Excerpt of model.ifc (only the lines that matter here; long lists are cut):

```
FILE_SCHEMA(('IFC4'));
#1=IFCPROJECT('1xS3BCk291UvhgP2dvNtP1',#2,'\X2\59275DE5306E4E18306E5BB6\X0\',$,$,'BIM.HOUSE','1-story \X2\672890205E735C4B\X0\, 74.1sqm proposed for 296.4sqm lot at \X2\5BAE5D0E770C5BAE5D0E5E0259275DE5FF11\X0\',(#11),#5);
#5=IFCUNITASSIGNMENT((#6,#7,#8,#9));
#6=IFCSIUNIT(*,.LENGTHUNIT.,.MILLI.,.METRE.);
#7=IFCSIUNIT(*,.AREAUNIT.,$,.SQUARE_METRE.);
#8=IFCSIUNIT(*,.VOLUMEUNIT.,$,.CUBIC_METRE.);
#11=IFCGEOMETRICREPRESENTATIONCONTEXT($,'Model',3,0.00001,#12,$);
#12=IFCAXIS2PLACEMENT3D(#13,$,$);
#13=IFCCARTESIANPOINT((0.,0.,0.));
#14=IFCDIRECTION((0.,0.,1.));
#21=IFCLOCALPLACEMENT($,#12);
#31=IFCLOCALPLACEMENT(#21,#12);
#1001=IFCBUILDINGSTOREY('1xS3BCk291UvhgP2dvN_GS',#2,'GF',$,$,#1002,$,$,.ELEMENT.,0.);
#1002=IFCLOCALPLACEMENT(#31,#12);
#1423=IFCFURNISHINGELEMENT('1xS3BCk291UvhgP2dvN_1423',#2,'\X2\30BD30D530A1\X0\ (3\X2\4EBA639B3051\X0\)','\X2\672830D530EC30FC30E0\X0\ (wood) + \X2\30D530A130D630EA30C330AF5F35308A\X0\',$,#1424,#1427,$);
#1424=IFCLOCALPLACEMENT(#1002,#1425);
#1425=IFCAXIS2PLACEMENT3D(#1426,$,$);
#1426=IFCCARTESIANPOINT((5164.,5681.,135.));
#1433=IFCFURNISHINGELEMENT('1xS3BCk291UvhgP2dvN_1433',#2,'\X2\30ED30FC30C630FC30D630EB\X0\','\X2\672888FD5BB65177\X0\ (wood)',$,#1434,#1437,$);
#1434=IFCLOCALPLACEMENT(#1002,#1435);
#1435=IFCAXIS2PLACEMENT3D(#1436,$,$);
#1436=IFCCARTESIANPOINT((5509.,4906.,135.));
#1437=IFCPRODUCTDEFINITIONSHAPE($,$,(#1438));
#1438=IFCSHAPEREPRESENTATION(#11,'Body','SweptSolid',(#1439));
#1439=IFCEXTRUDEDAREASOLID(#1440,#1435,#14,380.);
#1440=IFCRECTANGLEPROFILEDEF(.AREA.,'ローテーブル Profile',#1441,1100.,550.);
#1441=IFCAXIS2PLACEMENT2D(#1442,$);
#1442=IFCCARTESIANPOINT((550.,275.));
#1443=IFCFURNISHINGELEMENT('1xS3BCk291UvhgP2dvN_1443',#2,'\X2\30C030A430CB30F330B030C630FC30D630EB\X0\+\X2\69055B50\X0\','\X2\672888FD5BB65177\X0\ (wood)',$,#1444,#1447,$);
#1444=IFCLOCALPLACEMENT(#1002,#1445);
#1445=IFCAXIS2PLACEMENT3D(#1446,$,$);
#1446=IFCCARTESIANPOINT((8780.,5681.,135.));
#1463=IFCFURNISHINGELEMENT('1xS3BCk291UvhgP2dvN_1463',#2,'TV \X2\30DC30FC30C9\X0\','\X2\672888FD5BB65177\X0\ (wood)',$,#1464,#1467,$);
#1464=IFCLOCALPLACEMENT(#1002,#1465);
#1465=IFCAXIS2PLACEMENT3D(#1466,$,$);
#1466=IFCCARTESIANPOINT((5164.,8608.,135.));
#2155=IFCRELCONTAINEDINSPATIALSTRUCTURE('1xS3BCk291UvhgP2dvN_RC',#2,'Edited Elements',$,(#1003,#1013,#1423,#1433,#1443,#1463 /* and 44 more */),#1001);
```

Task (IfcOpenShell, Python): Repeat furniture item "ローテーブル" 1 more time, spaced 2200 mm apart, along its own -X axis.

```python
import ifcopenshell
import ifcopenshell.api.geometry
import ifcopenshell.api.root
import ifcopenshell.util.element
import ifcopenshell.util.placement

model = ifcopenshell.open("model.ifc")


def reuse_history(source, copy):
    """copy_class also copies each property set's owner history, people and application; keep the originals."""
    for rel in copy.IsDefinedBy:
        if rel.is_a("IfcRelDefinesByProperties") and (history := rel.RelatingPropertyDefinition.OwnerHistory):
            rel.RelatingPropertyDefinition.OwnerHistory = source.OwnerHistory
            ifcopenshell.util.element.remove_deep2(model, history)


source = model.by_id(1433)
base = ifcopenshell.util.placement.get_local_placement(source.ObjectPlacement)
step = -base[:3, 0] * 2200.0

for i in range(1, 2):
    copy = ifcopenshell.api.root.copy_class(model, product=source)
    copy.Representation = ifcopenshell.util.element.copy_deep(
        model, source.Representation, exclude=["IfcGeometricRepresentationContext", "IfcRepresentationMap"]
    )
    reuse_history(source, copy)
    matrix = base.copy()
    matrix[:3, 3] += i * step
    print("added at", matrix[:3, 3].round(3) + 0.0)
    ifcopenshell.api.geometry.edit_object_placement(model, product=copy, matrix=matrix, is_si=False)

model.write("model_rev.ifc")
```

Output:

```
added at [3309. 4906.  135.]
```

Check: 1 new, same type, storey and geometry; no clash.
